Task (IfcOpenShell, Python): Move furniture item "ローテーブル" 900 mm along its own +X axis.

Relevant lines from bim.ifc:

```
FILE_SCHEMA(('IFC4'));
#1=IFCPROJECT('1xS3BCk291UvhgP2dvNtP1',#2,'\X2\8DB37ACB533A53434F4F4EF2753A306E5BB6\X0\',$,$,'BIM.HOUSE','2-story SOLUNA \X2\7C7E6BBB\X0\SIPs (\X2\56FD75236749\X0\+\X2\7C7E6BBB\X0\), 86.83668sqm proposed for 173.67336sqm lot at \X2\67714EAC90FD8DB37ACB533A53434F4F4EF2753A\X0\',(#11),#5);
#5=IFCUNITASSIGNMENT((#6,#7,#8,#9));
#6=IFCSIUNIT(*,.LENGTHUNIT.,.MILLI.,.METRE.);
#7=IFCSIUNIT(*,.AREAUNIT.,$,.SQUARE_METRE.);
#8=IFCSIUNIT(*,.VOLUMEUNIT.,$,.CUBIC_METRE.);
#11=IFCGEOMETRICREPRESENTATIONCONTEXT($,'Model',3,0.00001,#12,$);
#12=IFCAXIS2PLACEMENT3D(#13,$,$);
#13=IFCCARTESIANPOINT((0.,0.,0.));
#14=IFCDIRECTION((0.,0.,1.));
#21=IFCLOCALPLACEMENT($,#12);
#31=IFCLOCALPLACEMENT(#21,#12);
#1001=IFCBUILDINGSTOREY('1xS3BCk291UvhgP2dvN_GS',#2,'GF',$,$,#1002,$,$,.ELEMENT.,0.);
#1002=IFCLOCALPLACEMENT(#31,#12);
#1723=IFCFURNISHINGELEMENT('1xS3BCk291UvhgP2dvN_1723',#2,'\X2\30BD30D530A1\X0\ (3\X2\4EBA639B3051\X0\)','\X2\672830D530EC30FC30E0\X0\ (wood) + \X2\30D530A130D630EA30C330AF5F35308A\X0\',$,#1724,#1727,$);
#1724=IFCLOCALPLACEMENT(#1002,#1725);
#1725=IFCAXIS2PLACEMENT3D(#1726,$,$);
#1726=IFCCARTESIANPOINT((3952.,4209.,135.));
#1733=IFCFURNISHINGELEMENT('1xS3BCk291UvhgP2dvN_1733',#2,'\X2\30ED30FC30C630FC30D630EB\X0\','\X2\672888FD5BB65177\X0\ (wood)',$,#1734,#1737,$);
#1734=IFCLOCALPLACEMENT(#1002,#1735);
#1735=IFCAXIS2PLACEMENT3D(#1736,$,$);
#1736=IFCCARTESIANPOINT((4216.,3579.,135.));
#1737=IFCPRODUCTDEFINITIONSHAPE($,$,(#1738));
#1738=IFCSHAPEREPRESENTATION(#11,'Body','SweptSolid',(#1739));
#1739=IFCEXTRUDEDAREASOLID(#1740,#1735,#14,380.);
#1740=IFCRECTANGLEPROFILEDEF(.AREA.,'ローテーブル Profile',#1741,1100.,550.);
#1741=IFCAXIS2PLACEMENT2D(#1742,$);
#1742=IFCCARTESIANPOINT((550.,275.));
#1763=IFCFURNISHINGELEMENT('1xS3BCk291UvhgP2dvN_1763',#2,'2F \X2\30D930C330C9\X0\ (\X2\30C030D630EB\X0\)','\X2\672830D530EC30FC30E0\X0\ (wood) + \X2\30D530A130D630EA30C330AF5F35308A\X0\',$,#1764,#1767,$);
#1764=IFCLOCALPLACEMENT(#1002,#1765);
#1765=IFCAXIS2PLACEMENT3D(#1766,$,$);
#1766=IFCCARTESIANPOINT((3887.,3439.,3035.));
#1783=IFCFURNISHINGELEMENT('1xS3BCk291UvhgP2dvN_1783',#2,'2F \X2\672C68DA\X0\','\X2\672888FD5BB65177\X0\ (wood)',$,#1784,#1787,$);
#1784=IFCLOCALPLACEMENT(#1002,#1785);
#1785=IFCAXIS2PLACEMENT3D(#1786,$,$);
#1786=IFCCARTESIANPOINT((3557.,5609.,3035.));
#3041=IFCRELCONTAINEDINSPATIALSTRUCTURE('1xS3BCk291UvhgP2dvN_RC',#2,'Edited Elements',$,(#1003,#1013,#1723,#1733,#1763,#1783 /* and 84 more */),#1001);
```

```python
import ifcopenshell
import ifcopenshell.api.geometry
import ifcopenshell.util.placement

model = ifcopenshell.open("bim.ifc")

item = model.by_guid("1xS3BCk291UvhgP2dvN_1733")
matrix = ifcopenshell.util.placement.get_local_placement(item.ObjectPlacement)
matrix[:3, 3] += matrix[:3, 0] * 900.0
ifcopenshell.api.geometry.edit_object_placement(model, product=item, matrix=matrix, is_si=False)

print(ifcopenshell.util.placement.get_local_placement(item.ObjectPlacement).round(3) + 0.0)

model.write("bim_v2.ifc")
```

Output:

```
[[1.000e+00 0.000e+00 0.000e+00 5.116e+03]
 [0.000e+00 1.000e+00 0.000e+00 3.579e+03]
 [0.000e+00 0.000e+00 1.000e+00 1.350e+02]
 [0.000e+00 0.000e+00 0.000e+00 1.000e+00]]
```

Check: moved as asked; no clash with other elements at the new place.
